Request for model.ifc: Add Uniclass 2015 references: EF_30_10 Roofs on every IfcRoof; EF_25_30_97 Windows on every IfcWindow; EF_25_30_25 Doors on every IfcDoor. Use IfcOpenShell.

First a look at what the model holds.

```python
import ifcopenshell

model = ifcopenshell.open("model.ifc")
print(model.schema)
print("classifications:", [c.Name for c in model.by_type("IfcClassification")])
for ifc_class in ("IfcDoor", "IfcRoof", "IfcStair", "IfcWall", "IfcWindow"):
    print(ifc_class, len(model.by_type(ifc_class)))
```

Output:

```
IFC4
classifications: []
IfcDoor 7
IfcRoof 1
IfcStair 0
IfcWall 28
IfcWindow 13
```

```python
import ifcopenshell
import ifcopenshell.api.classification

model = ifcopenshell.open("model.ifc")

system = ifcopenshell.api.classification.add_classification(model, classification="Uniclass 2015")

codes = {
    "IfcRoof": ("EF_30_10", "Roofs"),
    "IfcWindow": ("EF_25_30_97", "Windows"),
    "IfcDoor": ("EF_25_30_25", "Doors"),
}
for ifc_class, (code, name) in codes.items():
    products = model.by_type(ifc_class)
    ifcopenshell.api.classification.add_reference(
        model, products=products, classification=system, identification=code, name=name
    )
    print(code, len(products))

model.write("model_updated.ifc")
```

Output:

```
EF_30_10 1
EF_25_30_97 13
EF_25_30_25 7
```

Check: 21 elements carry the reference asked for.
